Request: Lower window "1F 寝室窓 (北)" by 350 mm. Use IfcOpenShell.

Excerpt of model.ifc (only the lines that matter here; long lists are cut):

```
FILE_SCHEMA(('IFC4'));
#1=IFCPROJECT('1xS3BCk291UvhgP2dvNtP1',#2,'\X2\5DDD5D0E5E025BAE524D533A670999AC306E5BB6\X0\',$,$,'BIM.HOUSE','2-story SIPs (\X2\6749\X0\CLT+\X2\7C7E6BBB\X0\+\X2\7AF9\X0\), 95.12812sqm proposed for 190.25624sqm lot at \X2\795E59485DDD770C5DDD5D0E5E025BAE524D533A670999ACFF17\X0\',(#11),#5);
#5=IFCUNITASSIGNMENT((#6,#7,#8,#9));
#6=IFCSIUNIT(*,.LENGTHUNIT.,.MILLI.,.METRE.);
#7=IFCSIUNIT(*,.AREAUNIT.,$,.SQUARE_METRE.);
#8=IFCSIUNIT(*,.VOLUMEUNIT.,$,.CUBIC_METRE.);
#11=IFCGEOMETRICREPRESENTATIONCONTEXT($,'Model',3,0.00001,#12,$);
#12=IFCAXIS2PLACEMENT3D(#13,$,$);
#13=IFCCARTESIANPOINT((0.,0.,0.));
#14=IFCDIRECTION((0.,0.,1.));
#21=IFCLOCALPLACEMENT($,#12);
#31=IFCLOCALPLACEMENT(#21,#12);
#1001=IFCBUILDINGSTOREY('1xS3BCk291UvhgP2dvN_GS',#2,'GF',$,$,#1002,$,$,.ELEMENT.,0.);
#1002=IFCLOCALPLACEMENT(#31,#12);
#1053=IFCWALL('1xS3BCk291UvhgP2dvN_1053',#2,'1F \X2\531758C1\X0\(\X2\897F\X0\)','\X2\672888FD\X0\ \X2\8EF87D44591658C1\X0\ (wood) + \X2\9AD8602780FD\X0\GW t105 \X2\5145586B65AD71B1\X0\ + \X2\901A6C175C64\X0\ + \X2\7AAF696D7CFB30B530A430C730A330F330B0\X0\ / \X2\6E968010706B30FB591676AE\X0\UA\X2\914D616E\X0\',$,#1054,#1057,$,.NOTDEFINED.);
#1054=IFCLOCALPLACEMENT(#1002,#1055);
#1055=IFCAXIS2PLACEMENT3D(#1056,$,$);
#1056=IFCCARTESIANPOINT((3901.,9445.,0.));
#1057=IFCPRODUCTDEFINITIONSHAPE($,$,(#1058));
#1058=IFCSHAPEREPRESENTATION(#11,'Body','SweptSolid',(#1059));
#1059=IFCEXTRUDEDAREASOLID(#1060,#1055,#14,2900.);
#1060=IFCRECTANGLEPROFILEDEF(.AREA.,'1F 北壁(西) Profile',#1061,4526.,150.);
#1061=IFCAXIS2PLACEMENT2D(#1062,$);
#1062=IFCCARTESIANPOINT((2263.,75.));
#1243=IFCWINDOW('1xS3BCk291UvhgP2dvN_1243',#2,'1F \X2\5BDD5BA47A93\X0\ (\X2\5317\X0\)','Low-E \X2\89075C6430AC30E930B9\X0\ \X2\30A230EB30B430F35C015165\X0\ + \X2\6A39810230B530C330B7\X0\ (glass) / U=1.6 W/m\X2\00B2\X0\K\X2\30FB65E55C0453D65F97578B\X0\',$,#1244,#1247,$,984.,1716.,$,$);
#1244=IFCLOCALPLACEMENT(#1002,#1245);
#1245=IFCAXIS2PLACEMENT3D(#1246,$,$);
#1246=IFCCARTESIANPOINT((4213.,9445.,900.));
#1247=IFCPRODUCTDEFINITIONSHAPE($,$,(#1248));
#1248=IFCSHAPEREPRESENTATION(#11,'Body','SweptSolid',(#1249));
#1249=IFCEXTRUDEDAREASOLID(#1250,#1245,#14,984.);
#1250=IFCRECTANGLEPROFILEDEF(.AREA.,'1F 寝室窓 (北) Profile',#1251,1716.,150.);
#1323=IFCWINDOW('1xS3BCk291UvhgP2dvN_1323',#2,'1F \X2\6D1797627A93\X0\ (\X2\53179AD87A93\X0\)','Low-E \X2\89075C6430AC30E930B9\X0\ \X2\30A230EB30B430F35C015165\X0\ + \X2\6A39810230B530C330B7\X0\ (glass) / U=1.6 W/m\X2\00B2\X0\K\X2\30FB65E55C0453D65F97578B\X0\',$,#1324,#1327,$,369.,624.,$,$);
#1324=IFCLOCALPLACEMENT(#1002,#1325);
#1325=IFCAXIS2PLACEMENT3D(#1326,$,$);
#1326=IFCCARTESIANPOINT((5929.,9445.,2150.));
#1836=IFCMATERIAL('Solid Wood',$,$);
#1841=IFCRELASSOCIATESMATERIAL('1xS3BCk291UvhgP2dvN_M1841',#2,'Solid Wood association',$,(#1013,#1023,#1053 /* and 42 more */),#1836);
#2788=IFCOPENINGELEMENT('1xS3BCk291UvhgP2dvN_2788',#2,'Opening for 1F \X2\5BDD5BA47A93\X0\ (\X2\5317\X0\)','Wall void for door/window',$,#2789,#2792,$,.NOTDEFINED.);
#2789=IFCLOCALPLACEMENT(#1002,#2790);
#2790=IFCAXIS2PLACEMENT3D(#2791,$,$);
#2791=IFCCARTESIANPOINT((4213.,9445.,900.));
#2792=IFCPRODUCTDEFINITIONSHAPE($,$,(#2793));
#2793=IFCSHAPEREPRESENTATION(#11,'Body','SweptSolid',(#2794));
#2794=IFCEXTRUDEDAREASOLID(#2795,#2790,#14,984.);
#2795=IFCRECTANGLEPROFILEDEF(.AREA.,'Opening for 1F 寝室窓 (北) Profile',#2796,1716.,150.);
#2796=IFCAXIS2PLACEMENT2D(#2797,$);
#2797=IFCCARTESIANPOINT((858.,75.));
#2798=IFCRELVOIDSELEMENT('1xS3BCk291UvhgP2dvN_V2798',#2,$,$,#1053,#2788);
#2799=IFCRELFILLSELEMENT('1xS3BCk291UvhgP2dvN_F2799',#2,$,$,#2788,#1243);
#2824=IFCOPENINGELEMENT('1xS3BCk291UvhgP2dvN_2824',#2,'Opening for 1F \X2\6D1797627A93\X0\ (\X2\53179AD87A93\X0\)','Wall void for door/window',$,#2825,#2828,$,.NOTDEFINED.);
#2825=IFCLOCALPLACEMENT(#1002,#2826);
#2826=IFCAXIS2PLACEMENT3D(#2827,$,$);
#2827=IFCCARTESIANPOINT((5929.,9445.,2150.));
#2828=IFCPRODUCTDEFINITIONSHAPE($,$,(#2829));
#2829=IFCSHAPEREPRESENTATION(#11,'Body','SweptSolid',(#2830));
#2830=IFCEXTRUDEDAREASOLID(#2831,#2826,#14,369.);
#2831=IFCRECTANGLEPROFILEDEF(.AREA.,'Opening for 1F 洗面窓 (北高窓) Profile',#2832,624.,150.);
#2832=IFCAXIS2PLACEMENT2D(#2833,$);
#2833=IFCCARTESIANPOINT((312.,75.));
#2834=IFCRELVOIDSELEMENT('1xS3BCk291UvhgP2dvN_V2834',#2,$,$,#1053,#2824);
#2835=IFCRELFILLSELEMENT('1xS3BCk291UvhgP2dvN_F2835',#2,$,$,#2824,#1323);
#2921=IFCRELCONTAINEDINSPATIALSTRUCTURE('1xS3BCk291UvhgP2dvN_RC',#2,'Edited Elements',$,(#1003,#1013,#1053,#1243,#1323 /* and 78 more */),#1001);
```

```python
import numpy as np
import ifcopenshell
import ifcopenshell.api.geometry
import ifcopenshell.util.placement
import ifcopenshell.util.unit

model = ifcopenshell.open("model.ifc")
unit_scale = ifcopenshell.util.unit.calculate_unit_scale(model)

window = model.by_guid("1xS3BCk291UvhgP2dvN_1243")
opening = window.FillsVoids[0].RelatingOpeningElement
dz = -0.35 / unit_scale

shift = np.array([0.0, 0.0, dz])
# The window is not placed relative to its opening, so move both.
for product in (opening, window):
    matrix = ifcopenshell.util.placement.get_local_placement(product.ObjectPlacement)
    matrix[:3, 3] += shift
    ifcopenshell.api.geometry.edit_object_placement(model, product=product, matrix=matrix, is_si=False)

print(f"moved by {dz * unit_scale:+.3f} m")

model.write("model_v2.ifc")
```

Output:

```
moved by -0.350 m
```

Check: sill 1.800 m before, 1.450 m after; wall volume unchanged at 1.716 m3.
